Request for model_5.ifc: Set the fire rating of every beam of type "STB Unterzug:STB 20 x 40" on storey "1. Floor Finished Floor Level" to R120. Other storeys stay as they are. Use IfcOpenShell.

First a look at what the model holds.

```python
import ifcopenshell
import ifcopenshell.util.element

model = ifcopenshell.open("model_5.ifc")
print(model.schema)
storey = next(s for s in model.by_type("IfcBuildingStorey") if s.Name == "1. Floor Finished Floor Level")
beams = [e for e in ifcopenshell.util.element.get_decomposition(storey) if e.is_a("IfcBeam")]
seen = {}
for e in beams:
    element_type = ifcopenshell.util.element.get_type(e)
    key = (element_type.Name if element_type != e and element_type else None, ifcopenshell.util.element.get_pset(e, "Pset_BeamCommon", "FireRating"))
    seen[key] = seen.get(key, 0) + 1
for (name, value), count in sorted(seen.items(), key=str):
    print(count, "x", name, "|", value)
```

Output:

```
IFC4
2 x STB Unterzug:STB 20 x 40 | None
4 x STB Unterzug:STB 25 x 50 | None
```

```python
import ifcopenshell
import ifcopenshell.api.pset
import ifcopenshell.util.element

model = ifcopenshell.open("model_5.ifc")

storey = next(s for s in model.by_type("IfcBuildingStorey") if s.Name == "1. Floor Finished Floor Level")
beams = [e for e in ifcopenshell.util.element.get_decomposition(storey) if e.is_a("IfcBeam")]

count = 0
for e in beams:
    element_type = ifcopenshell.util.element.get_type(e)
    if element_type in (None, e) or element_type.Name != "STB Unterzug:STB 20 x 40":
        continue
    # add_pset returns the element's existing set when there is one.
    pset = ifcopenshell.api.pset.add_pset(model, product=e, name="Pset_BeamCommon")
    ifcopenshell.api.pset.edit_pset(model, pset=pset, properties={"FireRating": "R120"})
    count += 1

print(count, "beams updated")

model.write("model_5_rev.ifc")
```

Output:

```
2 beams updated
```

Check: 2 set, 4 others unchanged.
